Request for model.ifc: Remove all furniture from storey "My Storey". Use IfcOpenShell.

First a look at what the model holds.

```python
import ifcopenshell
import ifcopenshell.util.element

model = ifcopenshell.open("model.ifc")
print(model.schema)
storey = next(s for s in model.by_type("IfcBuildingStorey") if s.Name == "My Storey")
furniture = [e for e in ifcopenshell.util.element.get_decomposition(storey) if e.is_a("IfcFurnishingElement")]
seen = {}
for e in furniture:
    element_type = ifcopenshell.util.element.get_type(e)
    name = element_type.Name if element_type not in (None, e) else None
    seen[name] = seen.get(name, 0) + 1
for name, count in sorted(seen.items(), key=str):
    print(count, "x", name)
```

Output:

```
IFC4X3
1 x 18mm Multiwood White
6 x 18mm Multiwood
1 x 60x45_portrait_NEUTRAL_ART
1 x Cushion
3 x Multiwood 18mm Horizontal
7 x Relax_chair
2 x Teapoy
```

```python
import ifcopenshell
import ifcopenshell.api.root
import ifcopenshell.util.element

model = ifcopenshell.open("model.ifc")

storey = next(s for s in model.by_type("IfcBuildingStorey") if s.Name == "My Storey")
furniture = [e for e in ifcopenshell.util.element.get_decomposition(storey) if e.is_a("IfcFurnishingElement")]

for e in furniture:
    ifcopenshell.api.root.remove_product(model, product=e)
print(len(furniture), "removed")

model.write("model_edited.ifc")
```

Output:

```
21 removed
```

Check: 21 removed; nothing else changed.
